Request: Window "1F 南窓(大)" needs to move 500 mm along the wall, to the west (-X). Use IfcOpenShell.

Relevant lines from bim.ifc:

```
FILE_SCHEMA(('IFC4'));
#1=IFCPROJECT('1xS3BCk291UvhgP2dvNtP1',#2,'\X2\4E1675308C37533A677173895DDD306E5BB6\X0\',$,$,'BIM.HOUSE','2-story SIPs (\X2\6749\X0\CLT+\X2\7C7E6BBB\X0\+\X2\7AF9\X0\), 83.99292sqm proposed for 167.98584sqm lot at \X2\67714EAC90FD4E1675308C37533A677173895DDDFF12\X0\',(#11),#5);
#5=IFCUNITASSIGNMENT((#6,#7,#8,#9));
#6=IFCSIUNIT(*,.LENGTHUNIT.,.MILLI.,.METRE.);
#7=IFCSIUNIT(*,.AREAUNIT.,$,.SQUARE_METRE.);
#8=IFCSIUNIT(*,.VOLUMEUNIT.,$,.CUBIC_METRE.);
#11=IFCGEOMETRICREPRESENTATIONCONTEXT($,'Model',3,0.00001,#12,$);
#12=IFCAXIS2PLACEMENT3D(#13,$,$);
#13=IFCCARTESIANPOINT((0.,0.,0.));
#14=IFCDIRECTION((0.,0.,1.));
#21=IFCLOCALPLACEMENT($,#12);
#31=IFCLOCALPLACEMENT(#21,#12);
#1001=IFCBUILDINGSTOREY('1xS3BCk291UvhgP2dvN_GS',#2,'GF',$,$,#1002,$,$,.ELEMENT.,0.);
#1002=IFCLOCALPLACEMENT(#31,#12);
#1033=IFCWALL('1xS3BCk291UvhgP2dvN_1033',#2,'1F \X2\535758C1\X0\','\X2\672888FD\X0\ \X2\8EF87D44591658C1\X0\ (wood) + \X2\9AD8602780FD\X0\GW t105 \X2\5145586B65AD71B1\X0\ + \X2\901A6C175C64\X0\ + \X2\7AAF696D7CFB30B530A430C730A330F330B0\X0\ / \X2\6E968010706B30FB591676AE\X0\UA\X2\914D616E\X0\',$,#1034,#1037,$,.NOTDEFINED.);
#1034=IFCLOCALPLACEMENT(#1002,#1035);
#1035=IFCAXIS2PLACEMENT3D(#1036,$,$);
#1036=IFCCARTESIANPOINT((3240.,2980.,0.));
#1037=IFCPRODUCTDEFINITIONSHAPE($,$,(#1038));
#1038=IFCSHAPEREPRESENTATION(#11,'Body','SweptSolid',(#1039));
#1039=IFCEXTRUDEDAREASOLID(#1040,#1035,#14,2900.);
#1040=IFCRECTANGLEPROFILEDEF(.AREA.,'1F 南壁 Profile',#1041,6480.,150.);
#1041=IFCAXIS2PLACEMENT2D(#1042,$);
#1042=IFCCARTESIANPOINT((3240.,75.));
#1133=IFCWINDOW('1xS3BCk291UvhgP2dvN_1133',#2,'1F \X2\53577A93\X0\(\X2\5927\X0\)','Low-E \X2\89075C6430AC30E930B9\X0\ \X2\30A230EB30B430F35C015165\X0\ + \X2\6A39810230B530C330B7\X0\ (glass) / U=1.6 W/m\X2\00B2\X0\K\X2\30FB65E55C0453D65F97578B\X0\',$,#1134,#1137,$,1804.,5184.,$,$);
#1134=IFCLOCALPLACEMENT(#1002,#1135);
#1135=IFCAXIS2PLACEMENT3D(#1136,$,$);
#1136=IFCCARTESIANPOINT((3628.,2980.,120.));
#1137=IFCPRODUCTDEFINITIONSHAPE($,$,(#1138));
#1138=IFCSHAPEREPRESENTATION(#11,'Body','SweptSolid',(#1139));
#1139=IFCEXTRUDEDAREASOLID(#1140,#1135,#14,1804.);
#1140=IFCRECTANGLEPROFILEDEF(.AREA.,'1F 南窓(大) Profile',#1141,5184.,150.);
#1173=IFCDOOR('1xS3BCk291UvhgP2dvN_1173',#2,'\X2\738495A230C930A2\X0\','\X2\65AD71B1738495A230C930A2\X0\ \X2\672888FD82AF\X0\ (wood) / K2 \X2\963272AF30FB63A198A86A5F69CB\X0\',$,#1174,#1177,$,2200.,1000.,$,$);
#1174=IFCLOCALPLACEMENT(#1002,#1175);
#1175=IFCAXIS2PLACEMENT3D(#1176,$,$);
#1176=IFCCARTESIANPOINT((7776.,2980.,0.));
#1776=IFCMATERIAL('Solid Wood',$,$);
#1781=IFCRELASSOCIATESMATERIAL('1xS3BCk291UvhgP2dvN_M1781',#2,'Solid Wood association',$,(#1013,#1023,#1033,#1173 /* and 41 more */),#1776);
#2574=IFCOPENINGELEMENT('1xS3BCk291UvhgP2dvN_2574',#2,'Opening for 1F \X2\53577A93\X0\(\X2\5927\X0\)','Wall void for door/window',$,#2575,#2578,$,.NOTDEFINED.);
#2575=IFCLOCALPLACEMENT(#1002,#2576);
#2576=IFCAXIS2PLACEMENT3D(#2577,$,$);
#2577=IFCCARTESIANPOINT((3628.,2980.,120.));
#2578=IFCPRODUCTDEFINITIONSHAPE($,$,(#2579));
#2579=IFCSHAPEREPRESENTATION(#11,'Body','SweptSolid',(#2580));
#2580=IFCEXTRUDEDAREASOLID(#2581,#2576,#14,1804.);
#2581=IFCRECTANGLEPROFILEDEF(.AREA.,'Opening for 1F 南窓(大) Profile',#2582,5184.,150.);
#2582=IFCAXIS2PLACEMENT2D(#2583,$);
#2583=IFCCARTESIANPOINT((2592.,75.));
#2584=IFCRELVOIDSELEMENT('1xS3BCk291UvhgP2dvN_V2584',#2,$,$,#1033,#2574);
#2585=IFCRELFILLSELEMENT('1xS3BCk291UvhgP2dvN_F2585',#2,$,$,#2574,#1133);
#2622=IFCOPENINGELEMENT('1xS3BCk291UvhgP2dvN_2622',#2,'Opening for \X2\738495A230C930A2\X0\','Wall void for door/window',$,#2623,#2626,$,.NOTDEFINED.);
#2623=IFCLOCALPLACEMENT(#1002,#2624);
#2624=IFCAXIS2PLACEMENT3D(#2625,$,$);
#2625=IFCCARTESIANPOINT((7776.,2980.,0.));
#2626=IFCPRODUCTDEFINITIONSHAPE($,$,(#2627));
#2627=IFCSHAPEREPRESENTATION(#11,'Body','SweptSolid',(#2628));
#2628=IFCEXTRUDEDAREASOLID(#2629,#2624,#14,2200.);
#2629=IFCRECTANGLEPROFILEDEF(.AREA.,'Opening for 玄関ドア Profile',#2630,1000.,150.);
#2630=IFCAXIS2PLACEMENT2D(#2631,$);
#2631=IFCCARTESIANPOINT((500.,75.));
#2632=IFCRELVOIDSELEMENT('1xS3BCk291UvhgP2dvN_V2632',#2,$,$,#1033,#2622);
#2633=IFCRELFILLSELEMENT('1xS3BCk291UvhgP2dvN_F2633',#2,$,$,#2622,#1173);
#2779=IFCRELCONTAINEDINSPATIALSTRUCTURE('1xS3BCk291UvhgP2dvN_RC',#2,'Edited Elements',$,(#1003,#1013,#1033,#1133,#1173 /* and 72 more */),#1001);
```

```python
import ifcopenshell
import ifcopenshell.api.geometry
import ifcopenshell.util.placement
import ifcopenshell.util.unit

model = ifcopenshell.open("bim.ifc")
unit_scale = ifcopenshell.util.unit.calculate_unit_scale(model)

window = model.by_guid("1xS3BCk291UvhgP2dvN_1133")
opening = window.FillsVoids[0].RelatingOpeningElement
wall = opening.VoidsElements[0].RelatingBuildingElement

wall_matrix = ifcopenshell.util.placement.get_local_placement(wall.ObjectPlacement)
shift = wall_matrix[:3, 0] * -0.5 / unit_scale
before = ifcopenshell.util.placement.get_local_placement(window.ObjectPlacement)[:3, 3].copy()

# The window is not placed relative to its opening, so move both.
for product in (opening, window):
    matrix = ifcopenshell.util.placement.get_local_placement(product.ObjectPlacement)
    matrix[:3, 3] += shift
    ifcopenshell.api.geometry.edit_object_placement(model, product=product, matrix=matrix, is_si=False)

after = ifcopenshell.util.placement.get_local_placement(window.ObjectPlacement)[:3, 3]
print("window moved by", (after - before).round(3) + 0.0)

model.write("bim_rev.ifc")
```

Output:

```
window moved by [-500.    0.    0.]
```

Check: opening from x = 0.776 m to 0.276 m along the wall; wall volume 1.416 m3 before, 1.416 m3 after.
